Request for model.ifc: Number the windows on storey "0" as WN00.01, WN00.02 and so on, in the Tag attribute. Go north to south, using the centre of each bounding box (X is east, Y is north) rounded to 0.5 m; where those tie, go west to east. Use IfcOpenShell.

First a look at what the model holds.

```python
import ifcopenshell
import ifcopenshell.util.element
import ifcopenshell.util.placement

model = ifcopenshell.open("model.ifc")
print(model.schema)
storey = next(s for s in model.by_type("IfcBuildingStorey") if s.Name == "0")
windows = [e for e in ifcopenshell.util.element.get_decomposition(storey) if e.is_a("IfcWindow")]
for e in sorted(windows, key=lambda e: e.id()):
    origin = ifcopenshell.util.placement.get_local_placement(e.ObjectPlacement)[:3, 3]
    print(e.id(), e.Tag, e.Name, origin.round(2) + 0.0, sep=" | ")
```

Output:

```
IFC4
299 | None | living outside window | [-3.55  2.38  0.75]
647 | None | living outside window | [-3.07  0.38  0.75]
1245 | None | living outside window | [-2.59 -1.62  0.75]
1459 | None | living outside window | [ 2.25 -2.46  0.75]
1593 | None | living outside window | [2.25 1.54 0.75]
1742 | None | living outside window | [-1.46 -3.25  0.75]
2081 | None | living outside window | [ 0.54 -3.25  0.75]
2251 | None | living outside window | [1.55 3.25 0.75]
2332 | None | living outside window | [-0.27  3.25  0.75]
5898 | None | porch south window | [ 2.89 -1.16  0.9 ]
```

```python
import ifcopenshell
import ifcopenshell.geom
import ifcopenshell.util.element
import ifcopenshell.util.shape

model = ifcopenshell.open("model.ifc")
settings = ifcopenshell.geom.settings()
settings.set("use-world-coords", True)


def centre(element):
    shape = ifcopenshell.geom.create_shape(settings, element)
    return ifcopenshell.util.shape.get_bbox_centroid(shape.geometry)


storey = next(s for s in model.by_type("IfcBuildingStorey") if s.Name == "0")
windows = [e for e in ifcopenshell.util.element.get_decomposition(storey) if e.is_a("IfcWindow")]

# Insertion points can sit at a corner or the storey origin, so sort by the geometry (in metres).
centres = {e: centre(e) for e in windows}
windows.sort(key=lambda e: (-round(centres[e][1] / 0.5), centres[e][0]))

for i, e in enumerate(windows, start=1):
    number = f"WN00.{i:02d}"
    e.Tag = number
    print(e.id(), number)

model.write("model_v2.ifc")
```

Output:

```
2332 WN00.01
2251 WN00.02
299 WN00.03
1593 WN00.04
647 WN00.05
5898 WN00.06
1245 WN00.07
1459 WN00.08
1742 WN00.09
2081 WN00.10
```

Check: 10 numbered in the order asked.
